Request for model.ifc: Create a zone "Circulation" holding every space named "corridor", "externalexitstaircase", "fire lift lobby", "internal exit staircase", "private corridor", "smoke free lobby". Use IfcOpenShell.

First a look at what the model holds.

```python
import ifcopenshell

model = ifcopenshell.open("model.ifc")
print(model.schema)
seen = {}
for space in model.by_type("IfcSpace"):
    seen[space.LongName] = seen.get(space.LongName, 0) + 1
for name, count in sorted(seen.items(), key=str):
    print(count, "x", name)
print("zones:", [z.Name for z in model.by_type("IfcZone")][:20])
```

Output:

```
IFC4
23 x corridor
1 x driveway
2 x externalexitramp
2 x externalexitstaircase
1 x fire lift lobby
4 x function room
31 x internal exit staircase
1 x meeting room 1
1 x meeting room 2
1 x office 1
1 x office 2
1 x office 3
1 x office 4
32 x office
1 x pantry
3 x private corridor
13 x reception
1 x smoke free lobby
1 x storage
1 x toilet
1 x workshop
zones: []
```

```python
import ifcopenshell
import ifcopenshell.api.group
import ifcopenshell.api.root

model = ifcopenshell.open("model.ifc")

names = {"corridor", "externalexitstaircase", "fire lift lobby", "internal exit staircase", "private corridor", "smoke free lobby"}
spaces = [s for s in model.by_type("IfcSpace") if s.LongName in names]

zone = ifcopenshell.api.root.create_entity(model, ifc_class="IfcZone", name="Circulation")
ifcopenshell.api.group.assign_group(model, products=spaces, group=zone)
print(len(spaces), "spaces in", zone.Name)

model.write("model_rev.ifc")
```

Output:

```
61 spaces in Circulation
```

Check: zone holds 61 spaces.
